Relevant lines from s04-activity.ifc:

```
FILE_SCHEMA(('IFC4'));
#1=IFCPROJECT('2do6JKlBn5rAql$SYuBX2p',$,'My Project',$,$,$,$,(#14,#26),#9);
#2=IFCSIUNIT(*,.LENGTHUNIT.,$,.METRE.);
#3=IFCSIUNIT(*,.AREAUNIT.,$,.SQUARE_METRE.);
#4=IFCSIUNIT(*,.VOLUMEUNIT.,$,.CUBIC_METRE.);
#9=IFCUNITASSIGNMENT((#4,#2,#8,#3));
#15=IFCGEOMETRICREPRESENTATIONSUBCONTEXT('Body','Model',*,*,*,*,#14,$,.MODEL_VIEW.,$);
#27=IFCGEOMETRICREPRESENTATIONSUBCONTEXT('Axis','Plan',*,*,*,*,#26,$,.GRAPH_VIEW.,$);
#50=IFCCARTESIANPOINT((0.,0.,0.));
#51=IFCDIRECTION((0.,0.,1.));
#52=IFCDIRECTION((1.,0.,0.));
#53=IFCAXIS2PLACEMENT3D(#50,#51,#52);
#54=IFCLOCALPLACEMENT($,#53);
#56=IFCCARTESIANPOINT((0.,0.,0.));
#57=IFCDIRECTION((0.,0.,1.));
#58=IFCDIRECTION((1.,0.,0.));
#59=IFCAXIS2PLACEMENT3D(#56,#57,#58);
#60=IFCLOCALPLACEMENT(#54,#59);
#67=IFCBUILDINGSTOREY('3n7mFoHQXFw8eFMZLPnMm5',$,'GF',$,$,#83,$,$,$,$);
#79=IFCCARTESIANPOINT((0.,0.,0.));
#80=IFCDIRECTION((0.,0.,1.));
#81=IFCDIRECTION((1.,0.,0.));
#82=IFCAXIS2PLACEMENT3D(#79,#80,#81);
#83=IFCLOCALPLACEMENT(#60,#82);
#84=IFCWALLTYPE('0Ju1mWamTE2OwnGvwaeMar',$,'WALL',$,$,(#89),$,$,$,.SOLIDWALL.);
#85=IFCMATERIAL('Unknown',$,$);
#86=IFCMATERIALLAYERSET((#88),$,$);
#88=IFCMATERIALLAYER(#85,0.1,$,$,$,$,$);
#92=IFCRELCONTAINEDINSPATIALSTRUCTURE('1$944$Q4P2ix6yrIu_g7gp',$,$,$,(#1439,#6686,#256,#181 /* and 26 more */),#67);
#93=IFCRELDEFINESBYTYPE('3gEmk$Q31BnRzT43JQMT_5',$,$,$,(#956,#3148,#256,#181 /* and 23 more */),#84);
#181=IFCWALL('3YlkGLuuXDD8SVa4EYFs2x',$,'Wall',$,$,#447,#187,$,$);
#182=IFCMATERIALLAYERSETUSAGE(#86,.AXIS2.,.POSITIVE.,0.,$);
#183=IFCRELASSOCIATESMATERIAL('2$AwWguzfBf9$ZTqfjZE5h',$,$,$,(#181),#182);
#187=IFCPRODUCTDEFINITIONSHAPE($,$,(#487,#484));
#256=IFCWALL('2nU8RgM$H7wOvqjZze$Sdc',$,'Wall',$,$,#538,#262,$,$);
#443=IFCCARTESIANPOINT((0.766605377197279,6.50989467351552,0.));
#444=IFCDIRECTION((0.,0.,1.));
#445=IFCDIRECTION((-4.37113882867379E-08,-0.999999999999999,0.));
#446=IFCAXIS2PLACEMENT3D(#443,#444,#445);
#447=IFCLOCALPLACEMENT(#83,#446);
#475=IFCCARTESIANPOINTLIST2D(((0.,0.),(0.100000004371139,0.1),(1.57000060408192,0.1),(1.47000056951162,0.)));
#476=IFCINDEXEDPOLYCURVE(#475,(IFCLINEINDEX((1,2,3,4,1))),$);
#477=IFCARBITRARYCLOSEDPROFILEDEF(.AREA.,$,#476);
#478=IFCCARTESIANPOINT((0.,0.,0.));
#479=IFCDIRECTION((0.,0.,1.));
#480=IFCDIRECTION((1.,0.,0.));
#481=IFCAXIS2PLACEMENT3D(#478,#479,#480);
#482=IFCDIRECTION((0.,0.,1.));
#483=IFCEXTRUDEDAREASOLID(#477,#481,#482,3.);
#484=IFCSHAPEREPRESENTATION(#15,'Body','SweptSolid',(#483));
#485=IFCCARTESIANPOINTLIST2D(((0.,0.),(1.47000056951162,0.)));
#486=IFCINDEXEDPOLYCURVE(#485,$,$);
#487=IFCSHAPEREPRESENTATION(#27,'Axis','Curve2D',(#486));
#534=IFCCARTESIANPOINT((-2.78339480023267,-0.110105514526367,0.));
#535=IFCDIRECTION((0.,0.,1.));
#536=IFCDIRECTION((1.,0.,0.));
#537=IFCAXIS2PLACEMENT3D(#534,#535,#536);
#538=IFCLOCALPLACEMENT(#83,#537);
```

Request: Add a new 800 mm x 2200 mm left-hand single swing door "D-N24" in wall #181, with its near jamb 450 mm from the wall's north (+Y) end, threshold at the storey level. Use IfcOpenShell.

```python
import numpy as np
import ifcopenshell
import ifcopenshell.api.feature
import ifcopenshell.api.geometry
import ifcopenshell.api.root
import ifcopenshell.api.spatial
import ifcopenshell.geom
import ifcopenshell.util.element
import ifcopenshell.util.placement
import ifcopenshell.util.representation
import ifcopenshell.util.shape
import ifcopenshell.util.unit

model = ifcopenshell.open("s04-activity.ifc")
unit_scale = ifcopenshell.util.unit.calculate_unit_scale(model)
settings = ifcopenshell.geom.settings()


def volume(element):
    """Net volume in cubic metres, openings subtracted."""
    shape = ifcopenshell.geom.create_shape(settings, element)
    return ifcopenshell.util.shape.get_volume(shape.geometry)


wall = model.by_guid("3YlkGLuuXDD8SVa4EYFs2x")
storey = ifcopenshell.util.element.get_container(wall, ifc_class="IfcBuildingStorey")
context = ifcopenshell.util.representation.get_context(model, "Model", "Body", "MODEL_VIEW")
before = volume(wall)

width, height, from_end, sill = 0.8, 2.2, 0.45, 0.0  # metres

# The wall runs along its own X axis, and the end named is its -X end.
wall_shape = ifcopenshell.geom.create_shape(settings, wall)
x, y, z = ifcopenshell.util.shape.get_vertices(wall_shape.geometry).T
start = x.min() + from_end
face, thickness = float(y.min()), float(y.max() - y.min())
wall_matrix = ifcopenshell.util.placement.get_local_placement(wall.ObjectPlacement)
level = ifcopenshell.util.placement.get_local_placement(storey.ObjectPlacement)[2, 3]


def in_wall(x, y):
    """Placement at x, y metres in the wall's axes, at sill height."""
    matrix = wall_matrix.copy()
    matrix[:, 3] = wall_matrix @ np.array([x / unit_scale, y / unit_scale, 0.0, 1.0])
    matrix[2, 3] = level + sill / unit_scale
    return matrix


# Opening: a box that overshoots both wall faces by 50 mm.
opening = ifcopenshell.api.root.create_entity(model, ifc_class="IfcOpeningElement", predefined_type="OPENING")
box = ifcopenshell.api.geometry.add_wall_representation(
    model, context=context, length=width, height=height, thickness=thickness + 0.1
)
ifcopenshell.api.geometry.assign_representation(model, product=opening, representation=box)
ifcopenshell.api.geometry.edit_object_placement(model, product=opening, matrix=in_wall(start, face - 0.05), is_si=False)
ifcopenshell.api.feature.add_feature(model, feature=opening, element=wall)

door = ifcopenshell.api.root.create_entity(model, ifc_class="IfcDoor", name="D-N24", predefined_type="DOOR")
door.OverallWidth, door.OverallHeight = width / unit_scale, height / unit_scale
door.OperationType = "SINGLE_SWING_LEFT"
body = ifcopenshell.api.geometry.add_door_representation(
    model,
    context=context,
    overall_width=door.OverallWidth,
    overall_height=door.OverallHeight,
    operation_type="SINGLE_SWING_LEFT",
    lining_properties={"LiningDepth": thickness / unit_scale, "ThresholdDepth": thickness / unit_scale},
)
ifcopenshell.api.geometry.assign_representation(model, product=door, representation=body)
ifcopenshell.api.spatial.assign_container(model, products=[door], relating_structure=storey)
ifcopenshell.api.feature.add_filling(model, opening=opening, element=door)

# The lining spans the wall, so the door starts at the wall face.
ifcopenshell.api.geometry.edit_object_placement(model, product=door, matrix=in_wall(start, face), is_si=False)

after = volume(wall)

print(f"wall volume {before:.3f} -> {after:.3f} m3")

model.write("s04-activity_rev.ifc")
```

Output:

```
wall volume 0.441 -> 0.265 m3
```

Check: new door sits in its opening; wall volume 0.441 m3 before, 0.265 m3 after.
